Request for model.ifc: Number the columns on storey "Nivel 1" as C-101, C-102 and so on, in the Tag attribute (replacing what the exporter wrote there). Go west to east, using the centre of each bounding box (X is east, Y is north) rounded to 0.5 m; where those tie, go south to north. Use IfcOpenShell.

First a look at what the model holds.

```python
import ifcopenshell
import ifcopenshell.util.element
import ifcopenshell.util.placement

model = ifcopenshell.open("model.ifc")
print(model.schema)
storey = next(s for s in model.by_type("IfcBuildingStorey") if s.Name == "Nivel 1")
columns = [e for e in ifcopenshell.util.element.get_decomposition(storey) if e.is_a("IfcColumn")]
for e in sorted(columns, key=lambda e: e.id()):
    origin = ifcopenshell.util.placement.get_local_placement(e.ObjectPlacement)[:3, 3]
    print(e.id(), e.Tag, e.Name, origin.round(2) + 0.0, sep=" | ")
```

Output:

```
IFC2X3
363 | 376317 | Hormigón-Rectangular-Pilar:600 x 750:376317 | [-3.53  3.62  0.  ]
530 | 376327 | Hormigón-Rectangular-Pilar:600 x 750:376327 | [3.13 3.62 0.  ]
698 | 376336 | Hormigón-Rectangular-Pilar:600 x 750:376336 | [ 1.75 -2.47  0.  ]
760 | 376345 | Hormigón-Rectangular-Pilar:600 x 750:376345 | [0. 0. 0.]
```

```python
import ifcopenshell
import ifcopenshell.geom
import ifcopenshell.util.element
import ifcopenshell.util.shape

model = ifcopenshell.open("model.ifc")
settings = ifcopenshell.geom.settings()
settings.set("use-world-coords", True)


def centre(element):
    shape = ifcopenshell.geom.create_shape(settings, element)
    return ifcopenshell.util.shape.get_bbox_centroid(shape.geometry)


storey = next(s for s in model.by_type("IfcBuildingStorey") if s.Name == "Nivel 1")
columns = [e for e in ifcopenshell.util.element.get_decomposition(storey) if e.is_a("IfcColumn")]

# Insertion points can sit at a corner or the storey origin, so sort by the geometry (in metres).
centres = {e: centre(e) for e in columns}
columns.sort(key=lambda e: (round(centres[e][0] / 0.5), centres[e][1]))

for i, e in enumerate(columns, start=1):
    number = f"C-1{i:02d}"
    e.Tag = number
    print(e.id(), number)

model.write("model_updated.ifc")
```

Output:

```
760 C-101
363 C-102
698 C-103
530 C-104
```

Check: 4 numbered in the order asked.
